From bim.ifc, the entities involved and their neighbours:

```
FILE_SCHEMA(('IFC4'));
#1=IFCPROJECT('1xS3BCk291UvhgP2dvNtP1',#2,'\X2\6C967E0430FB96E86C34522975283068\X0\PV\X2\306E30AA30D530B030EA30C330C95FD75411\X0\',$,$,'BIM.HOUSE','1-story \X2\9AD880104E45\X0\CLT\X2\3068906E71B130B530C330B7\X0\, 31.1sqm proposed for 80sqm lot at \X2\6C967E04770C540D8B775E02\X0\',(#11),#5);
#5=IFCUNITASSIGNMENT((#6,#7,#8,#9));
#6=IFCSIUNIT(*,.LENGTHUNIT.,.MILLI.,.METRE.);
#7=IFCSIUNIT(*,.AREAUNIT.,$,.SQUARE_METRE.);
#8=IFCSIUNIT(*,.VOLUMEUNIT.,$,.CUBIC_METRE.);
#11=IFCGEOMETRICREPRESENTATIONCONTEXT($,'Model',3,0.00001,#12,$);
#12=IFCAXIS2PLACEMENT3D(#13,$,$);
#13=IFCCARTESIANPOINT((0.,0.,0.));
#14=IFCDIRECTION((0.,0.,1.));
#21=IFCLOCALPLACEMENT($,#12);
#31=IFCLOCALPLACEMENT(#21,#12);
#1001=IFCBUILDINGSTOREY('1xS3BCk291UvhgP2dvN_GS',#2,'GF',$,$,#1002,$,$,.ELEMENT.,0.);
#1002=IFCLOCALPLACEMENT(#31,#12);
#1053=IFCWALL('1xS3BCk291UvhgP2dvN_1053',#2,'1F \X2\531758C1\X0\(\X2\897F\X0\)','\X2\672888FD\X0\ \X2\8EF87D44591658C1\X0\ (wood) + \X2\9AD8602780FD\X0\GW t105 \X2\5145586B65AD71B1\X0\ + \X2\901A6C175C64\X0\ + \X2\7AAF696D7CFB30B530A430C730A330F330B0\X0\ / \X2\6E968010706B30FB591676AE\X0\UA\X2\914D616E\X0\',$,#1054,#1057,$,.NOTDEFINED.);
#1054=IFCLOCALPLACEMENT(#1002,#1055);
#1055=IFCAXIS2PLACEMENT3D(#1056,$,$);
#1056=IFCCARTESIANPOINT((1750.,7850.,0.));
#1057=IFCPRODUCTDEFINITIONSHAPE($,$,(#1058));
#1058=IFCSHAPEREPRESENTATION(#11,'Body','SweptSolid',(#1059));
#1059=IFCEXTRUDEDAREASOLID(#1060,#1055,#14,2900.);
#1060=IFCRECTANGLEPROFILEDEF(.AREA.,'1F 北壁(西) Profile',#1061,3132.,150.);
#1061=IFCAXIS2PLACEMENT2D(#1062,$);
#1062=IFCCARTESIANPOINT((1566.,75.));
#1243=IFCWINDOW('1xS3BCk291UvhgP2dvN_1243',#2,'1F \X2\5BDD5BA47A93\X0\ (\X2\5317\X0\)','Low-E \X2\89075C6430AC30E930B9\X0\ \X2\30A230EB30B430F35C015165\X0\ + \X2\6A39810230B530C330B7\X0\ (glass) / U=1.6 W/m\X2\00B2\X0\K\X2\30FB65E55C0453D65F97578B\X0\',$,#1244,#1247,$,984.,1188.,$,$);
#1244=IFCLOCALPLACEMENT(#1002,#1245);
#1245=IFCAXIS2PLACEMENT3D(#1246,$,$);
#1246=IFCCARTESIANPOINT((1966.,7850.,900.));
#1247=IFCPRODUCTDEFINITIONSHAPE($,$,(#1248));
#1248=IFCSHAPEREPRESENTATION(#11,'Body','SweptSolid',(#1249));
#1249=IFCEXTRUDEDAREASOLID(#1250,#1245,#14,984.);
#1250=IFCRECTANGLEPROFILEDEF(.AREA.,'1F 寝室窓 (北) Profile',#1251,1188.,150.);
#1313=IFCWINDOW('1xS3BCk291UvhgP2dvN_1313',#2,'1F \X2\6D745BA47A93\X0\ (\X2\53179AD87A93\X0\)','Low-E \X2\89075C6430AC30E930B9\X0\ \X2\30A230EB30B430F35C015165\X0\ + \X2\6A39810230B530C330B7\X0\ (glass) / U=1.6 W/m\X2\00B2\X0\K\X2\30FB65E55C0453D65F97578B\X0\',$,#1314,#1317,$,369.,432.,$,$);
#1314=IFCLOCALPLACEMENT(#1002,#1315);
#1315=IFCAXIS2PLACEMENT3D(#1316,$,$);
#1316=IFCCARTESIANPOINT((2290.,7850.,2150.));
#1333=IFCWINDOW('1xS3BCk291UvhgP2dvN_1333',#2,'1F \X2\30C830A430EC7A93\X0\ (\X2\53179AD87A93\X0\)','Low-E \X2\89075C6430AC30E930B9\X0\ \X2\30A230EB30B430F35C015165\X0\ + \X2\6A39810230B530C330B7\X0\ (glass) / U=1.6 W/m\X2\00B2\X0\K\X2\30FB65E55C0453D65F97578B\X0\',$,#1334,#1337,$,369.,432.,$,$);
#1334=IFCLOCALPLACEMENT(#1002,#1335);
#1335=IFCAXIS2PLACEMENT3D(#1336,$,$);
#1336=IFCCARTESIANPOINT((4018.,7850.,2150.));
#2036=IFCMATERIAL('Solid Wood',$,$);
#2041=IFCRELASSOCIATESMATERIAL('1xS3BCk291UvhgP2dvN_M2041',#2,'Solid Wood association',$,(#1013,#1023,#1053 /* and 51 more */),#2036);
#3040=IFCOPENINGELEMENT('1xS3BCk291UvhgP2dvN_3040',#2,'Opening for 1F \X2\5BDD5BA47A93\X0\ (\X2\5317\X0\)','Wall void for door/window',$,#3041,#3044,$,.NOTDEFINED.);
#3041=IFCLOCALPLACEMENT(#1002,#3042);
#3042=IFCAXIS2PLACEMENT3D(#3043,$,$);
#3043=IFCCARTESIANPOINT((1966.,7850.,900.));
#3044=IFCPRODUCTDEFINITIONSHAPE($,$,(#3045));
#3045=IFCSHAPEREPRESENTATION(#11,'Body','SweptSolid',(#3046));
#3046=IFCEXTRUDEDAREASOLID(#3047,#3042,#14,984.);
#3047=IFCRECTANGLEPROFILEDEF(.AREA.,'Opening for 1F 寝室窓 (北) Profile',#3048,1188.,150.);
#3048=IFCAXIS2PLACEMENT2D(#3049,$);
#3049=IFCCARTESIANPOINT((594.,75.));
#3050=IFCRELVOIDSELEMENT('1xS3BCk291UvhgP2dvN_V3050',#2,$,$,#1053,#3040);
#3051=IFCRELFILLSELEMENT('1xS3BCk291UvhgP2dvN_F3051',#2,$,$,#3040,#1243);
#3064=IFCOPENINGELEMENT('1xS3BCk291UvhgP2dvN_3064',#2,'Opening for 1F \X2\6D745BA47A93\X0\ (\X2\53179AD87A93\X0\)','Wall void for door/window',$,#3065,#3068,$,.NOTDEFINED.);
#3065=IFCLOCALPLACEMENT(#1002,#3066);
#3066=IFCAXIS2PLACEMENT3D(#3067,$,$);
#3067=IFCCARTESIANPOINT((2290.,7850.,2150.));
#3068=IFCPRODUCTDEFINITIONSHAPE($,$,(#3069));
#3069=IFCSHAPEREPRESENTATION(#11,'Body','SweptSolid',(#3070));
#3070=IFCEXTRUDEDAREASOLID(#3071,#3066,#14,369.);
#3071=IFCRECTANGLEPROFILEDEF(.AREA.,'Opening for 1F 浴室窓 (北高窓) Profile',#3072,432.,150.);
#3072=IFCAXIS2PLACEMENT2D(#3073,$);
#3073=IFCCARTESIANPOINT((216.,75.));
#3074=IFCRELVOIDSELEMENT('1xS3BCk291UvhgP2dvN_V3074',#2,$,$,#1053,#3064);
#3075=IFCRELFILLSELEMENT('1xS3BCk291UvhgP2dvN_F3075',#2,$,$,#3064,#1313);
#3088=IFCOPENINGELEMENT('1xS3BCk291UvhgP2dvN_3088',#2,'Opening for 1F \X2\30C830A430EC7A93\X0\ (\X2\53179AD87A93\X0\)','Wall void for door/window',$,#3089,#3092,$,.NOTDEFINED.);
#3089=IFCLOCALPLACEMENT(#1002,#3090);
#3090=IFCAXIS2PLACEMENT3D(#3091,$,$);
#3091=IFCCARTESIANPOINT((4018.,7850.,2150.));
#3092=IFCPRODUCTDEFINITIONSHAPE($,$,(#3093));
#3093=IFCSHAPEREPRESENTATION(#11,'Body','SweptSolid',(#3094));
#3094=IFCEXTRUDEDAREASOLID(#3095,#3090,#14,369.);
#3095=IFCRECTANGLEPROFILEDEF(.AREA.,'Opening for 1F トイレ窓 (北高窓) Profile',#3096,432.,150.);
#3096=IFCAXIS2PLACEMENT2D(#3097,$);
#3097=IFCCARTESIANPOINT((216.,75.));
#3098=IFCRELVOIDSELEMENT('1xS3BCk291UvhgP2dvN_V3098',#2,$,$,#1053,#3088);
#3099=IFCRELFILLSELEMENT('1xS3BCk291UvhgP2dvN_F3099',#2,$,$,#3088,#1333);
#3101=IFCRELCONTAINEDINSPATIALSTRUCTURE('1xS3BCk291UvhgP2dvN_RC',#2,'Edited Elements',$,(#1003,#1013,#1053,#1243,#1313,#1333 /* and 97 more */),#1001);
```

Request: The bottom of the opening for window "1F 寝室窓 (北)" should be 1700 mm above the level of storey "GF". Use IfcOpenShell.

```python
import numpy as np
import ifcopenshell
import ifcopenshell.api.geometry
import ifcopenshell.geom
import ifcopenshell.util.element
import ifcopenshell.util.placement
import ifcopenshell.util.shape
import ifcopenshell.util.unit

model = ifcopenshell.open("bim.ifc")
unit_scale = ifcopenshell.util.unit.calculate_unit_scale(model)

window = model.by_id(1243)
opening = window.FillsVoids[0].RelatingOpeningElement
storey = ifcopenshell.util.element.get_container(window, ifc_class="IfcBuildingStorey")
level = ifcopenshell.util.placement.get_local_placement(storey.ObjectPlacement)[2, 3]

# The opening's origin need not be at the sill, so measure its lowest point.
shape = ifcopenshell.geom.create_shape(ifcopenshell.geom.settings(), opening)
bottom = ifcopenshell.util.shape.get_shape_bottom_elevation(shape, shape.geometry) / unit_scale
dz = level + 1.7 / unit_scale - bottom

shift = np.array([0.0, 0.0, dz])
# The window is not placed relative to its opening, so move both.
for product in (opening, window):
    matrix = ifcopenshell.util.placement.get_local_placement(product.ObjectPlacement)
    matrix[:3, 3] += shift
    ifcopenshell.api.geometry.edit_object_placement(model, product=product, matrix=matrix, is_si=False)

print(f"moved by {dz * unit_scale:+.3f} m")

model.write("bim_updated.ifc")
```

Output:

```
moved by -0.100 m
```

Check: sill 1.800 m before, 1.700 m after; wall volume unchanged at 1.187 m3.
